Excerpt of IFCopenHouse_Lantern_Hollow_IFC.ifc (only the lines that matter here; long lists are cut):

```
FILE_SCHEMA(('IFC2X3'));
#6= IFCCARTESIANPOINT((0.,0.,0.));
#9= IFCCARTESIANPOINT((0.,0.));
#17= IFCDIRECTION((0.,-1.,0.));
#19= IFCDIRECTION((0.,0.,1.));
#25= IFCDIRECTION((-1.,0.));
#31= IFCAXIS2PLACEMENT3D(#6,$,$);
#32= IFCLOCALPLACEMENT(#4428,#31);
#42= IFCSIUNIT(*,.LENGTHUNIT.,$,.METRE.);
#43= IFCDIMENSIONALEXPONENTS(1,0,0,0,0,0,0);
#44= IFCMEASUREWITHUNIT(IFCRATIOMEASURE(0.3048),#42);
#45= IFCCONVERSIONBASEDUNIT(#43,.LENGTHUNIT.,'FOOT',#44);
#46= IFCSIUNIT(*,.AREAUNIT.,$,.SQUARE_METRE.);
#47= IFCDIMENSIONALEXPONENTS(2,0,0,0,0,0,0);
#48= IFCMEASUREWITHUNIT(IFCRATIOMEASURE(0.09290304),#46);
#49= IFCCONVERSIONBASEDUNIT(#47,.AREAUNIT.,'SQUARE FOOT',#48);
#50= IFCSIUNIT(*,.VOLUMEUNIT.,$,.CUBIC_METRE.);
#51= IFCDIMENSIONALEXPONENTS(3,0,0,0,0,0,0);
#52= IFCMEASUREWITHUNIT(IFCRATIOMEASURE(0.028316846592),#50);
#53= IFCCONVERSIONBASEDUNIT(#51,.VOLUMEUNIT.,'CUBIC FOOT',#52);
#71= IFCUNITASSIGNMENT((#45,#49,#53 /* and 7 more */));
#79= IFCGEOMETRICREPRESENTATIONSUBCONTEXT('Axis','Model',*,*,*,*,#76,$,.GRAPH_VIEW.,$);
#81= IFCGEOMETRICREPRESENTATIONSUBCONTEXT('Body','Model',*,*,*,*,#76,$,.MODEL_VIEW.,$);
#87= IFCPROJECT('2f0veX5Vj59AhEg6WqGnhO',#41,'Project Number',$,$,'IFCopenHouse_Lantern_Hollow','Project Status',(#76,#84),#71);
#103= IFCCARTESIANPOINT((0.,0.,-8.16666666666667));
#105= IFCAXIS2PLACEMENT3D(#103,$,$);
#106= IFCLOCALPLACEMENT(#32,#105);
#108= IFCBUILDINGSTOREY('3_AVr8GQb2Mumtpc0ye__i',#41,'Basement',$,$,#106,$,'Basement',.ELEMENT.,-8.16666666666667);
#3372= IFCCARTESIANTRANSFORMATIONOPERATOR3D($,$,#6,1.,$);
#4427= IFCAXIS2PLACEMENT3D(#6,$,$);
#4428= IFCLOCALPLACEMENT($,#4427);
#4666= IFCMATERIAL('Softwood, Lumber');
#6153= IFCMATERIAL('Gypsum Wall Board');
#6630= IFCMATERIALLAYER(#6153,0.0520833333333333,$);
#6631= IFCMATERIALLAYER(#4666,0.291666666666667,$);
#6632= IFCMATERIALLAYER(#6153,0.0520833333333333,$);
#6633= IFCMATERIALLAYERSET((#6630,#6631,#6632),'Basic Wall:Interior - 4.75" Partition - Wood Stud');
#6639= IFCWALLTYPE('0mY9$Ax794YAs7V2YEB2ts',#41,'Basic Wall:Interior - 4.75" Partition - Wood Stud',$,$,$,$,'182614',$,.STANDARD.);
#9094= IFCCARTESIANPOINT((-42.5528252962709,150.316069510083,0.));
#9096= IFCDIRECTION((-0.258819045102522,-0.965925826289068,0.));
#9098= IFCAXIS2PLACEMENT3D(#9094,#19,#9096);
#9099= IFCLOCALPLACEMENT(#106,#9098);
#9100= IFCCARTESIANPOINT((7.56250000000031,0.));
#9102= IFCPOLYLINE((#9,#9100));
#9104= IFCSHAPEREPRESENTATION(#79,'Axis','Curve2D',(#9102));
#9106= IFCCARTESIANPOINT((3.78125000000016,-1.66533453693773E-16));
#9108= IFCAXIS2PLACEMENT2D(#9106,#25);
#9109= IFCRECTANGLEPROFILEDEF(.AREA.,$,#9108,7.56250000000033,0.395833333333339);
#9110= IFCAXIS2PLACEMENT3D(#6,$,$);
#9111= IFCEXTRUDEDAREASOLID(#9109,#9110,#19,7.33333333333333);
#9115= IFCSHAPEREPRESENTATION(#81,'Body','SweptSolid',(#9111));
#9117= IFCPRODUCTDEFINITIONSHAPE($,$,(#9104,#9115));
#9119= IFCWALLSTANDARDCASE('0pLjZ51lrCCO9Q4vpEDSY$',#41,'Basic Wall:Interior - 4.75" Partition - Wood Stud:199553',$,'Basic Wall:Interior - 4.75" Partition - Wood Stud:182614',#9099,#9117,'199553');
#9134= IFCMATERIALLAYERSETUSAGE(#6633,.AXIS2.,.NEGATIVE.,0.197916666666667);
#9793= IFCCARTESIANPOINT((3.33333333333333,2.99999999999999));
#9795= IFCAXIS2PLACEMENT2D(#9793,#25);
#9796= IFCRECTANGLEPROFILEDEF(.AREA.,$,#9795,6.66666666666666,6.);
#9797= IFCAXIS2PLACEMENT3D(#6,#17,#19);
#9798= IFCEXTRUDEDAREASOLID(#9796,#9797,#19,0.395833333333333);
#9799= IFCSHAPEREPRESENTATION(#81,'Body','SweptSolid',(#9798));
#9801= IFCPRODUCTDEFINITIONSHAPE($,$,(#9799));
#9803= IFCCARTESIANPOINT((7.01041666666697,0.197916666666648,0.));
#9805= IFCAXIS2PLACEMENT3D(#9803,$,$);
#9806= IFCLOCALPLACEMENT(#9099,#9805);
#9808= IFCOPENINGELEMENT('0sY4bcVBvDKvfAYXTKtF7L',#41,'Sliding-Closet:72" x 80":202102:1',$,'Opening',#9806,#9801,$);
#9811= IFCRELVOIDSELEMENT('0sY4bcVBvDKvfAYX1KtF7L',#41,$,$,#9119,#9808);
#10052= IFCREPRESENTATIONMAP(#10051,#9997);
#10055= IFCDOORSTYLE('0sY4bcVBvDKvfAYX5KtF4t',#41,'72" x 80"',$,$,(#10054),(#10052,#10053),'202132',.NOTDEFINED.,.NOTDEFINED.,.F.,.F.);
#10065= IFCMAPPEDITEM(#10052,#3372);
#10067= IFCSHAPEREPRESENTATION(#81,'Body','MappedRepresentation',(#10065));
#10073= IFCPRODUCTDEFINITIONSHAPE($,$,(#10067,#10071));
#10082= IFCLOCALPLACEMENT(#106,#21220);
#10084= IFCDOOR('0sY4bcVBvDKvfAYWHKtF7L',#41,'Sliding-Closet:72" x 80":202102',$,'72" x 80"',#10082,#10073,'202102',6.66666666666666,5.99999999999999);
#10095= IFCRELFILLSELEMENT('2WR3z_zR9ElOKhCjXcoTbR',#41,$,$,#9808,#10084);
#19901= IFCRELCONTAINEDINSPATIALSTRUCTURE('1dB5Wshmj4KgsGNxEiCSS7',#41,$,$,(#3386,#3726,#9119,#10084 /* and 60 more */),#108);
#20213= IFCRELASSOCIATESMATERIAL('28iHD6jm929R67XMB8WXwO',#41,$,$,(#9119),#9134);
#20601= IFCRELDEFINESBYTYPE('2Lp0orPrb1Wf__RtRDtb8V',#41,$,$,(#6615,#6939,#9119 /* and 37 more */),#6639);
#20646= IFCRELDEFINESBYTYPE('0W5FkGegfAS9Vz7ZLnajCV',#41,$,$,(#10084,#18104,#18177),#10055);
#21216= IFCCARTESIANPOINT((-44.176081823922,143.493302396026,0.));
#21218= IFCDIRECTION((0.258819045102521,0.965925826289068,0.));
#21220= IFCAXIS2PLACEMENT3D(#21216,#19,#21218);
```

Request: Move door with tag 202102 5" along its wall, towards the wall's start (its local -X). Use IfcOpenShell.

```python
import ifcopenshell
import ifcopenshell.api.geometry
import ifcopenshell.util.placement
import ifcopenshell.util.unit

model = ifcopenshell.open("IFCopenHouse_Lantern_Hollow_IFC.ifc")
unit_scale = ifcopenshell.util.unit.calculate_unit_scale(model)

door = model.by_id(10084)
opening = door.FillsVoids[0].RelatingOpeningElement
wall = opening.VoidsElements[0].RelatingBuildingElement

wall_matrix = ifcopenshell.util.placement.get_local_placement(wall.ObjectPlacement)
shift = wall_matrix[:3, 0] * -5 * 0.0254 / unit_scale
before = ifcopenshell.util.placement.get_local_placement(door.ObjectPlacement)[:3, 3].copy()

# The door is not placed relative to its opening, so move both.
for product in (opening, door):
    matrix = ifcopenshell.util.placement.get_local_placement(product.ObjectPlacement)
    matrix[:3, 3] += shift
    ifcopenshell.api.geometry.edit_object_placement(model, product=product, matrix=matrix, is_si=False)

after = ifcopenshell.util.placement.get_local_placement(door.ObjectPlacement)[:3, 3]
print("door moved by", (after - before).round(3) + 0.0)

model.write("IFCopenHouse_Lantern_Hollow_IFC_rev.ifc")
```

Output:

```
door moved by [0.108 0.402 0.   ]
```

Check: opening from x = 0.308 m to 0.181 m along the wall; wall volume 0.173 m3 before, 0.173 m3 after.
